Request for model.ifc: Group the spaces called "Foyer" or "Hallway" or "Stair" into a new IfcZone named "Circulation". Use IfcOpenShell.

First a look at what the model holds.

```python
import ifcopenshell

model = ifcopenshell.open("model.ifc")
print(model.schema)
seen = {}
for space in model.by_type("IfcSpace"):
    seen[space.LongName] = seen.get(space.LongName, 0) + 1
for name, count in sorted(seen.items(), key=str):
    print(count, "x", name)
print("zones:", [z.Name for z in model.by_type("IfcZone")][:20])
```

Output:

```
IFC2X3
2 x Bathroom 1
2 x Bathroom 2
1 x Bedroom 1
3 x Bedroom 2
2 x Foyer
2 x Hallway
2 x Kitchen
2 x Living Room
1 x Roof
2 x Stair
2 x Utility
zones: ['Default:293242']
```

```python
import ifcopenshell
import ifcopenshell.api.group
import ifcopenshell.api.root

model = ifcopenshell.open("model.ifc")

names = {"Foyer", "Hallway", "Stair"}
spaces = [s for s in model.by_type("IfcSpace") if s.LongName in names]

zone = ifcopenshell.api.root.create_entity(model, ifc_class="IfcZone", name="Circulation")
ifcopenshell.api.group.assign_group(model, products=spaces, group=zone)
print(len(spaces), "spaces in", zone.Name)

model.write("model-out.ifc")
```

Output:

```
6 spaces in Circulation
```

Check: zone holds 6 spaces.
